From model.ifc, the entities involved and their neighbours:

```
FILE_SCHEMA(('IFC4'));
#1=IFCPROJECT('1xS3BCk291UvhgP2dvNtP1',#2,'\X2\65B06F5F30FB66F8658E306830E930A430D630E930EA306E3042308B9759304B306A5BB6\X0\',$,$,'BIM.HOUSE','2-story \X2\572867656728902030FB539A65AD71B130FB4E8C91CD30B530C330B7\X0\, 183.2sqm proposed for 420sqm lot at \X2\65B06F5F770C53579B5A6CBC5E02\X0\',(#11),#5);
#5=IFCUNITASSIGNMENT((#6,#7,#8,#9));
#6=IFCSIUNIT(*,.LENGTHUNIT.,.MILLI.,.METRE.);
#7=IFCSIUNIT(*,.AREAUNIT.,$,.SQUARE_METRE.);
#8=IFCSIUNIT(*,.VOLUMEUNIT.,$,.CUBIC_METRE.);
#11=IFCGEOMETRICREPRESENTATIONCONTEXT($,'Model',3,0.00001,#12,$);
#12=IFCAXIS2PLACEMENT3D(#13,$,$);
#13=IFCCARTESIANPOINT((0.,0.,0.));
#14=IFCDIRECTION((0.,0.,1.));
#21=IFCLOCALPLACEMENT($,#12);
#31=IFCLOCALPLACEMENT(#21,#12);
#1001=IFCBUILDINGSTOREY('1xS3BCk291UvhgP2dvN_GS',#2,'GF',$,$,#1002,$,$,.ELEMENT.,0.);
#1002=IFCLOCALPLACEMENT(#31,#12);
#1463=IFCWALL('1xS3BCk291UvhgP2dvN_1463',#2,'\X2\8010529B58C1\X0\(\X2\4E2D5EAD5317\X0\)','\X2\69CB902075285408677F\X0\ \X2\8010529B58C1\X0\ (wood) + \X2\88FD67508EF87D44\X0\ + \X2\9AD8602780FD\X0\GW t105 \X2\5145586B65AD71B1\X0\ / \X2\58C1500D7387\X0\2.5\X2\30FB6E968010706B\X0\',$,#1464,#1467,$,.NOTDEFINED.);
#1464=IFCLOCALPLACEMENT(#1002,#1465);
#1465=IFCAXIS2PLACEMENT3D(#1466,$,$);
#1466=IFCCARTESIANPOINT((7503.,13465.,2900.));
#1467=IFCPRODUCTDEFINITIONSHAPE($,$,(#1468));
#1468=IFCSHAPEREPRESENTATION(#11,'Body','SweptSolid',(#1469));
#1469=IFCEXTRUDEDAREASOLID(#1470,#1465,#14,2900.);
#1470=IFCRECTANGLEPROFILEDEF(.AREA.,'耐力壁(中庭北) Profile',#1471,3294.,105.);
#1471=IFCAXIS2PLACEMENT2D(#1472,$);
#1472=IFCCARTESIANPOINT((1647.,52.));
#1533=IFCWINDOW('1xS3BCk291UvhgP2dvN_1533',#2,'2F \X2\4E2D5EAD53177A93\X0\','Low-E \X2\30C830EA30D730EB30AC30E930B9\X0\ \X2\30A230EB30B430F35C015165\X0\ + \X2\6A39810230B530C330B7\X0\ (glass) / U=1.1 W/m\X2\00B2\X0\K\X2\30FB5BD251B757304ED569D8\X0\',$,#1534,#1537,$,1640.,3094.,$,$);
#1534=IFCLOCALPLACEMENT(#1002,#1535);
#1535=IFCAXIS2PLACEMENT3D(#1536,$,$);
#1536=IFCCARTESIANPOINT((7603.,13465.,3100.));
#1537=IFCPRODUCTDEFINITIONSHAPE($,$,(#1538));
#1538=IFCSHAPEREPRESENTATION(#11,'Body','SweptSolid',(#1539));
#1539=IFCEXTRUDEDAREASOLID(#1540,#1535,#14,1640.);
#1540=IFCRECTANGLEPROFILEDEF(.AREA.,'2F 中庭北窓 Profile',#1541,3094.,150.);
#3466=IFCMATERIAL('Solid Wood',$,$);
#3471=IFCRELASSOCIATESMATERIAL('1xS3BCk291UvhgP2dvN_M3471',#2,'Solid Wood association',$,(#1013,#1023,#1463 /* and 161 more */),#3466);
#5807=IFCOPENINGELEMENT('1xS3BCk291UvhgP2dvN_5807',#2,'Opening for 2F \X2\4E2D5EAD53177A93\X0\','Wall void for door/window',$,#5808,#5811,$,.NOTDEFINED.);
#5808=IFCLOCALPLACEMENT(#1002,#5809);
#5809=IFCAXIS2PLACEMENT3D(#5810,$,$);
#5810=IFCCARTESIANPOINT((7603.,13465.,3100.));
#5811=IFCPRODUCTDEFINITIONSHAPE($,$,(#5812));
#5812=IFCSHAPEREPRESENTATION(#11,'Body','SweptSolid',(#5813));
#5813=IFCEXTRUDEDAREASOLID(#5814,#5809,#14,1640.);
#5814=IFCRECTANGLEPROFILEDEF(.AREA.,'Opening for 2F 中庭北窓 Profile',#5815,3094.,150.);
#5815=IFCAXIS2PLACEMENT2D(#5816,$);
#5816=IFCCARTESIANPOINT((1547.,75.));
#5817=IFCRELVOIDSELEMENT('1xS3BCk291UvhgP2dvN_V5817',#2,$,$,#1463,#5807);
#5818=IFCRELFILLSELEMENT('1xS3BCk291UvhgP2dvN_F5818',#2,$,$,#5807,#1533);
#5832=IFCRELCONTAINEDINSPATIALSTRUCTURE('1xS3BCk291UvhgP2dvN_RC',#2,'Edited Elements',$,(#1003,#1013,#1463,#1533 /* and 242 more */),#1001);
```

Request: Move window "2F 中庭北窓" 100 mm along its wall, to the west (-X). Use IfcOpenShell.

```python
import ifcopenshell
import ifcopenshell.api.geometry
import ifcopenshell.util.placement

model = ifcopenshell.open("model.ifc")

window = model.by_guid("1xS3BCk291UvhgP2dvN_1533")
opening = window.FillsVoids[0].RelatingOpeningElement
wall = opening.VoidsElements[0].RelatingBuildingElement

wall_matrix = ifcopenshell.util.placement.get_local_placement(wall.ObjectPlacement)
shift = wall_matrix[:3, 0] * -100.0
before = ifcopenshell.util.placement.get_local_placement(window.ObjectPlacement)[:3, 3].copy()

# The window is not placed relative to its opening, so move both.
for product in (opening, window):
    matrix = ifcopenshell.util.placement.get_local_placement(product.ObjectPlacement)
    matrix[:3, 3] += shift
    ifcopenshell.api.geometry.edit_object_placement(model, product=product, matrix=matrix, is_si=False)

after = ifcopenshell.util.placement.get_local_placement(window.ObjectPlacement)[:3, 3]
print("window moved by", (after - before).round(3) + 0.0)

model.write("model_rev.ifc")
```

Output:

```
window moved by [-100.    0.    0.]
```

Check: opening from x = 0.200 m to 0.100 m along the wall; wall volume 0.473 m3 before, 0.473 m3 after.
